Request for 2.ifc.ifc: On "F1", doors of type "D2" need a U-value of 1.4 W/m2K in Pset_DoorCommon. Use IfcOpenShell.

First a look at what the model holds.

```python
import ifcopenshell
import ifcopenshell.util.element

model = ifcopenshell.open("2.ifc.ifc")
print(model.schema)
storey = next(s for s in model.by_type("IfcBuildingStorey") if s.Name == "F1")
doors = [e for e in ifcopenshell.util.element.get_decomposition(storey) if e.is_a("IfcDoor")]
seen = {}
for e in doors:
    element_type = ifcopenshell.util.element.get_type(e)
    key = (element_type.Name if element_type != e and element_type else None, ifcopenshell.util.element.get_pset(e, "Pset_DoorCommon", "ThermalTransmittance"))
    seen[key] = seen.get(key, 0) + 1
for (name, value), count in sorted(seen.items(), key=str):
    print(count, "x", name, "|", value)
```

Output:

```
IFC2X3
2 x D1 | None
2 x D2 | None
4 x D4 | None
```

```python
import ifcopenshell
import ifcopenshell.api.pset
import ifcopenshell.util.element

model = ifcopenshell.open("2.ifc.ifc")

storey = next(s for s in model.by_type("IfcBuildingStorey") if s.Name == "F1")
doors = [e for e in ifcopenshell.util.element.get_decomposition(storey) if e.is_a("IfcDoor")]

count = 0
for e in doors:
    element_type = ifcopenshell.util.element.get_type(e)
    if element_type in (None, e) or element_type.Name != "D2":
        continue
    # add_pset returns the element's existing set when there is one.
    pset = ifcopenshell.api.pset.add_pset(model, product=e, name="Pset_DoorCommon")
    ifcopenshell.api.pset.edit_pset(model, pset=pset, properties={"ThermalTransmittance": 1.4})
    count += 1

print(count, "doors updated")

model.write("2.ifc-out.ifc")
```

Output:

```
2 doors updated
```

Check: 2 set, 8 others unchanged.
